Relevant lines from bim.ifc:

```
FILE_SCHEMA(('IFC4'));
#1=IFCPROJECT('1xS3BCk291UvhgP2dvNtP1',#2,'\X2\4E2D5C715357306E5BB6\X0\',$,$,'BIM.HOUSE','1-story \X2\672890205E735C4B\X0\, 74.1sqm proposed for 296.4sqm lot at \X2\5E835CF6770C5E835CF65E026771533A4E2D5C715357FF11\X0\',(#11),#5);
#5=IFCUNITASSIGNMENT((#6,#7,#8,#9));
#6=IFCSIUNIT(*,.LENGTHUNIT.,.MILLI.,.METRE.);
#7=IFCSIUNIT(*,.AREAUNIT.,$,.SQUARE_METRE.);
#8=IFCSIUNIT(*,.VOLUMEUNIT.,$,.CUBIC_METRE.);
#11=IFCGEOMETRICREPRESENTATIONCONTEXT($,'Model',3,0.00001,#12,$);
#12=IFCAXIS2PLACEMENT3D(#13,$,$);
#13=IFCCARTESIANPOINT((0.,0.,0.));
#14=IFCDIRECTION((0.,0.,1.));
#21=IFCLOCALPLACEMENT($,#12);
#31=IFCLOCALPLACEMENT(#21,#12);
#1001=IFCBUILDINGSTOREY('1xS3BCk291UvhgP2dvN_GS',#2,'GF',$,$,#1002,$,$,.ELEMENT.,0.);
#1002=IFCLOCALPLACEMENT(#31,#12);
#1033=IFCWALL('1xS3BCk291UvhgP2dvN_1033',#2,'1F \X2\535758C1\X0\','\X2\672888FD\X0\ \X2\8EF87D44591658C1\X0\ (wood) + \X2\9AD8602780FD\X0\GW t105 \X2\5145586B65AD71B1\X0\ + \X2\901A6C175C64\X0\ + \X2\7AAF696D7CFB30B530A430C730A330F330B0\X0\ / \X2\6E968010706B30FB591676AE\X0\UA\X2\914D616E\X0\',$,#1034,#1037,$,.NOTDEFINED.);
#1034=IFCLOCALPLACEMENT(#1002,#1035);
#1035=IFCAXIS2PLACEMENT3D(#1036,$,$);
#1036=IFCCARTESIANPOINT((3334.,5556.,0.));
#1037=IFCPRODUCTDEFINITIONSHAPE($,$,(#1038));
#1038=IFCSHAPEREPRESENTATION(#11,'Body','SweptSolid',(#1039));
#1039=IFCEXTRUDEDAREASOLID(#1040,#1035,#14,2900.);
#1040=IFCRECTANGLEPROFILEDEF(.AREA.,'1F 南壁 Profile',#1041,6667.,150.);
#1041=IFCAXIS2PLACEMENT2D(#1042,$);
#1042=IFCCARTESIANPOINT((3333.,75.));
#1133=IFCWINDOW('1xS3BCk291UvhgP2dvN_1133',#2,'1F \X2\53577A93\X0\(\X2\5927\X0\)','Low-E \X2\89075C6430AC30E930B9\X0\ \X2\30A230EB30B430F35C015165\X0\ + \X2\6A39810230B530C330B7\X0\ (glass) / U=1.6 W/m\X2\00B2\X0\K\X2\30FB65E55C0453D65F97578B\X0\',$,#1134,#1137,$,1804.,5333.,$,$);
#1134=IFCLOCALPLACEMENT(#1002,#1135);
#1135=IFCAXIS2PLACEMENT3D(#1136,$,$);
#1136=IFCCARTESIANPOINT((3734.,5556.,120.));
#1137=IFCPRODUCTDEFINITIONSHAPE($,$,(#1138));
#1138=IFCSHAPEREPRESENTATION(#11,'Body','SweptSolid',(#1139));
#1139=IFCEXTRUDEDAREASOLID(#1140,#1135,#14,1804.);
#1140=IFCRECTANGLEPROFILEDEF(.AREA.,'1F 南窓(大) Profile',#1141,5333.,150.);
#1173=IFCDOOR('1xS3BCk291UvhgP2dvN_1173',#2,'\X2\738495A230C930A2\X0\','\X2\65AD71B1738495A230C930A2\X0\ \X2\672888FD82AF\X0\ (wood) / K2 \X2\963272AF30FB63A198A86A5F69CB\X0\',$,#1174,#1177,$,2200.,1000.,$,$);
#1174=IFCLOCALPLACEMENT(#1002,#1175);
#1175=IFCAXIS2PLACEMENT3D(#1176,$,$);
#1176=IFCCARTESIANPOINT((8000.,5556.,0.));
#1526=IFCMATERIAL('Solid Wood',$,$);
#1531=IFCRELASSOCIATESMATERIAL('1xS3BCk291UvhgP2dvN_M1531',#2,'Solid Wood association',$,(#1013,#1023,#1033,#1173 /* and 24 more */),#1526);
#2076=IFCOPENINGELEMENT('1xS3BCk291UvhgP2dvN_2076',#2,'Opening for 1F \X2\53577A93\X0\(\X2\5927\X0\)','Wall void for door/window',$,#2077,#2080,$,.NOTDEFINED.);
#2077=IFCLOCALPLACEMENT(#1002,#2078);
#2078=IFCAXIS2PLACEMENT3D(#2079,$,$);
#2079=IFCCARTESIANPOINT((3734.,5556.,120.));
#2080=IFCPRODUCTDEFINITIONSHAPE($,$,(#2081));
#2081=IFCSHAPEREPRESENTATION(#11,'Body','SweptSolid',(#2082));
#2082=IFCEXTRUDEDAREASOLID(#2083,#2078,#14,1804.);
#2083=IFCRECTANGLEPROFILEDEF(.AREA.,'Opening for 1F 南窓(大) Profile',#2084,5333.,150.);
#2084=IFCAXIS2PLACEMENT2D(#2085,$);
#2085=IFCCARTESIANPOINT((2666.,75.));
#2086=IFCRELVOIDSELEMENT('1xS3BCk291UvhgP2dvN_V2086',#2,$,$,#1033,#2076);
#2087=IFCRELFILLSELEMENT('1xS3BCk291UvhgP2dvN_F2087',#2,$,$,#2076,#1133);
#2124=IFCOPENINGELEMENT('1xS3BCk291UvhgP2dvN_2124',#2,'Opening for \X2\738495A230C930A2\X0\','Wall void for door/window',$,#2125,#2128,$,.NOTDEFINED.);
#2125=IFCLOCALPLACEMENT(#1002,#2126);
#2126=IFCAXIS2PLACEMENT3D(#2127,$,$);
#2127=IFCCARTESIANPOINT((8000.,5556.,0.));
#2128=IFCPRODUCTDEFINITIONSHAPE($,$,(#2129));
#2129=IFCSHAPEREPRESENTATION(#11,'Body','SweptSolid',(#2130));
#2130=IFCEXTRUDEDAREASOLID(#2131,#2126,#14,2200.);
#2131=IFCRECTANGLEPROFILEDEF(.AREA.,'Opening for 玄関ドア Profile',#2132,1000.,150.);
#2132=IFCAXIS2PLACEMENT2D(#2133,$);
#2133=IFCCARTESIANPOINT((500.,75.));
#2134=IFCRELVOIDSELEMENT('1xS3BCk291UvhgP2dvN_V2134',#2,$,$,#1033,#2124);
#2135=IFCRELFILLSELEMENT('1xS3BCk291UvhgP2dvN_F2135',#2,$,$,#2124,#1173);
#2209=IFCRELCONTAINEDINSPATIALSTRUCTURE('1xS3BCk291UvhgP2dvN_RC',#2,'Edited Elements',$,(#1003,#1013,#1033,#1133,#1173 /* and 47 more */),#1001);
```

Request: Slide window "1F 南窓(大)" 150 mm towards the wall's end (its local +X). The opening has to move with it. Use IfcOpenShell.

```python
import ifcopenshell
import ifcopenshell.api.geometry
import ifcopenshell.util.placement

model = ifcopenshell.open("bim.ifc")

window = model.by_guid("1xS3BCk291UvhgP2dvN_1133")
opening = window.FillsVoids[0].RelatingOpeningElement
wall = opening.VoidsElements[0].RelatingBuildingElement

wall_matrix = ifcopenshell.util.placement.get_local_placement(wall.ObjectPlacement)
shift = wall_matrix[:3, 0] * 150.0
before = ifcopenshell.util.placement.get_local_placement(window.ObjectPlacement)[:3, 3].copy()

# The window is not placed relative to its opening, so move both.
for product in (opening, window):
    matrix = ifcopenshell.util.placement.get_local_placement(product.ObjectPlacement)
    matrix[:3, 3] += shift
    ifcopenshell.api.geometry.edit_object_placement(model, product=product, matrix=matrix, is_si=False)

after = ifcopenshell.util.placement.get_local_placement(window.ObjectPlacement)[:3, 3]
print("window moved by", (after - before).round(3) + 0.0)

model.write("bim-out.ifc")
```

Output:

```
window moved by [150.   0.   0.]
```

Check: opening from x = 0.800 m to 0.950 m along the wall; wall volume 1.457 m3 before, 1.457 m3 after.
